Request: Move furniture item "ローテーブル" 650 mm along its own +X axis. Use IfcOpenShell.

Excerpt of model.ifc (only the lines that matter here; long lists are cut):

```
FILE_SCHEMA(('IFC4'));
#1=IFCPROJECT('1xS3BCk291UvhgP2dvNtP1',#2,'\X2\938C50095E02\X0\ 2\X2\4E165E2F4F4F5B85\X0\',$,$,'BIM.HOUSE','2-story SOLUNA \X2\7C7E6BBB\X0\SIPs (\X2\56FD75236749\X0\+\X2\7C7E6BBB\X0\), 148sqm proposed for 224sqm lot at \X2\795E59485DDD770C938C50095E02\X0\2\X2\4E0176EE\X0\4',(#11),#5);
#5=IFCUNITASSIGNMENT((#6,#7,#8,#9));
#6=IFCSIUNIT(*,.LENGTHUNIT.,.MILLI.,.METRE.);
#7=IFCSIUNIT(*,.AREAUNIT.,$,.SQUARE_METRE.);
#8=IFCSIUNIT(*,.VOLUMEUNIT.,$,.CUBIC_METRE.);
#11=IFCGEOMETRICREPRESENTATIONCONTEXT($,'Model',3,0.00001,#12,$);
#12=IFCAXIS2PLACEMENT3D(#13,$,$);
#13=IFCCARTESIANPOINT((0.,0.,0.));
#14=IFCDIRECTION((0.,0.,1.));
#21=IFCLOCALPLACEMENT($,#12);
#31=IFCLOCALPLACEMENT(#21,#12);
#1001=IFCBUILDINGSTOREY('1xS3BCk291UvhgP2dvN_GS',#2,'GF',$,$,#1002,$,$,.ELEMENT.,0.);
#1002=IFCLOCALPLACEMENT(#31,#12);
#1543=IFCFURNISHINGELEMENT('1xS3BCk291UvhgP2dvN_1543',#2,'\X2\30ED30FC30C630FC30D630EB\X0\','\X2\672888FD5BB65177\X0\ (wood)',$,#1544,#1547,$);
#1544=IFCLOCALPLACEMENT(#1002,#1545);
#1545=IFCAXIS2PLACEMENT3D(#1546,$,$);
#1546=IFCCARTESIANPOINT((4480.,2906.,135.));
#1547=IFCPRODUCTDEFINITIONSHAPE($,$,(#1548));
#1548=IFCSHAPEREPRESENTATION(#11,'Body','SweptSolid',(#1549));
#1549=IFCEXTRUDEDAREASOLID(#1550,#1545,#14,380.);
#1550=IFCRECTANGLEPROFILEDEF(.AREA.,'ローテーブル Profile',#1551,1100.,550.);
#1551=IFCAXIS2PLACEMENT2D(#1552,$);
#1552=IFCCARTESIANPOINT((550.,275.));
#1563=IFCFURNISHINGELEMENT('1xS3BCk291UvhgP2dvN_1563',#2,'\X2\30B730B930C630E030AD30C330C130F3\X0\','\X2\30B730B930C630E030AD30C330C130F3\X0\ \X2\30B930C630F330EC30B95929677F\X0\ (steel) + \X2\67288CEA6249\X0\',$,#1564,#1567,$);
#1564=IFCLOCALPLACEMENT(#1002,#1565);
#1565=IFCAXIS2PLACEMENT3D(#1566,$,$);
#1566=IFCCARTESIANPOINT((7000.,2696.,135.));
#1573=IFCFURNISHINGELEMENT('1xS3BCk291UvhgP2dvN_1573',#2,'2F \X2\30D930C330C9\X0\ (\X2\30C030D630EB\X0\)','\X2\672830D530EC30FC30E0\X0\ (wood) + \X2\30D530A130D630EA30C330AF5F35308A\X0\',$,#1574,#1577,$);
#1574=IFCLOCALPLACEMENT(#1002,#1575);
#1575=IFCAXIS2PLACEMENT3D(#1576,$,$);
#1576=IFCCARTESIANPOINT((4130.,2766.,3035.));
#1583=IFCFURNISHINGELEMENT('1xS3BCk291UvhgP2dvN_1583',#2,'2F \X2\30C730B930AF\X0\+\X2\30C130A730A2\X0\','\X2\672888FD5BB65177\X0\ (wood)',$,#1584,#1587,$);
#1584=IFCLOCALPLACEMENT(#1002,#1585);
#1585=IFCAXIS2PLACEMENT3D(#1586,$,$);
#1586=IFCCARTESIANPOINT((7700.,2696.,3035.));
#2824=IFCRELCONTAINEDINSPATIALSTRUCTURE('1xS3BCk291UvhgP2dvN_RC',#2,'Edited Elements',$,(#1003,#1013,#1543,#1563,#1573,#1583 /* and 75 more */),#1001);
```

```python
import ifcopenshell
import ifcopenshell.api.geometry
import ifcopenshell.util.placement
import ifcopenshell.util.unit

model = ifcopenshell.open("model.ifc")
unit_scale = ifcopenshell.util.unit.calculate_unit_scale(model)

item = model.by_guid("1xS3BCk291UvhgP2dvN_1543")
matrix = ifcopenshell.util.placement.get_local_placement(item.ObjectPlacement)
matrix[:3, 3] += matrix[:3, 0] * 0.65 / unit_scale
ifcopenshell.api.geometry.edit_object_placement(model, product=item, matrix=matrix, is_si=False)

print(ifcopenshell.util.placement.get_local_placement(item.ObjectPlacement).round(3) + 0.0)

model.write("model_edited.ifc")
```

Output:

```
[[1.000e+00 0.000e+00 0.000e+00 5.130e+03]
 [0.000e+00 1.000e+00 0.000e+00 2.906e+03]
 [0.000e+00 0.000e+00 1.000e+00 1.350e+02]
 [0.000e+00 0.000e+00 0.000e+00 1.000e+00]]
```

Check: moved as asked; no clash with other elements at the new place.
